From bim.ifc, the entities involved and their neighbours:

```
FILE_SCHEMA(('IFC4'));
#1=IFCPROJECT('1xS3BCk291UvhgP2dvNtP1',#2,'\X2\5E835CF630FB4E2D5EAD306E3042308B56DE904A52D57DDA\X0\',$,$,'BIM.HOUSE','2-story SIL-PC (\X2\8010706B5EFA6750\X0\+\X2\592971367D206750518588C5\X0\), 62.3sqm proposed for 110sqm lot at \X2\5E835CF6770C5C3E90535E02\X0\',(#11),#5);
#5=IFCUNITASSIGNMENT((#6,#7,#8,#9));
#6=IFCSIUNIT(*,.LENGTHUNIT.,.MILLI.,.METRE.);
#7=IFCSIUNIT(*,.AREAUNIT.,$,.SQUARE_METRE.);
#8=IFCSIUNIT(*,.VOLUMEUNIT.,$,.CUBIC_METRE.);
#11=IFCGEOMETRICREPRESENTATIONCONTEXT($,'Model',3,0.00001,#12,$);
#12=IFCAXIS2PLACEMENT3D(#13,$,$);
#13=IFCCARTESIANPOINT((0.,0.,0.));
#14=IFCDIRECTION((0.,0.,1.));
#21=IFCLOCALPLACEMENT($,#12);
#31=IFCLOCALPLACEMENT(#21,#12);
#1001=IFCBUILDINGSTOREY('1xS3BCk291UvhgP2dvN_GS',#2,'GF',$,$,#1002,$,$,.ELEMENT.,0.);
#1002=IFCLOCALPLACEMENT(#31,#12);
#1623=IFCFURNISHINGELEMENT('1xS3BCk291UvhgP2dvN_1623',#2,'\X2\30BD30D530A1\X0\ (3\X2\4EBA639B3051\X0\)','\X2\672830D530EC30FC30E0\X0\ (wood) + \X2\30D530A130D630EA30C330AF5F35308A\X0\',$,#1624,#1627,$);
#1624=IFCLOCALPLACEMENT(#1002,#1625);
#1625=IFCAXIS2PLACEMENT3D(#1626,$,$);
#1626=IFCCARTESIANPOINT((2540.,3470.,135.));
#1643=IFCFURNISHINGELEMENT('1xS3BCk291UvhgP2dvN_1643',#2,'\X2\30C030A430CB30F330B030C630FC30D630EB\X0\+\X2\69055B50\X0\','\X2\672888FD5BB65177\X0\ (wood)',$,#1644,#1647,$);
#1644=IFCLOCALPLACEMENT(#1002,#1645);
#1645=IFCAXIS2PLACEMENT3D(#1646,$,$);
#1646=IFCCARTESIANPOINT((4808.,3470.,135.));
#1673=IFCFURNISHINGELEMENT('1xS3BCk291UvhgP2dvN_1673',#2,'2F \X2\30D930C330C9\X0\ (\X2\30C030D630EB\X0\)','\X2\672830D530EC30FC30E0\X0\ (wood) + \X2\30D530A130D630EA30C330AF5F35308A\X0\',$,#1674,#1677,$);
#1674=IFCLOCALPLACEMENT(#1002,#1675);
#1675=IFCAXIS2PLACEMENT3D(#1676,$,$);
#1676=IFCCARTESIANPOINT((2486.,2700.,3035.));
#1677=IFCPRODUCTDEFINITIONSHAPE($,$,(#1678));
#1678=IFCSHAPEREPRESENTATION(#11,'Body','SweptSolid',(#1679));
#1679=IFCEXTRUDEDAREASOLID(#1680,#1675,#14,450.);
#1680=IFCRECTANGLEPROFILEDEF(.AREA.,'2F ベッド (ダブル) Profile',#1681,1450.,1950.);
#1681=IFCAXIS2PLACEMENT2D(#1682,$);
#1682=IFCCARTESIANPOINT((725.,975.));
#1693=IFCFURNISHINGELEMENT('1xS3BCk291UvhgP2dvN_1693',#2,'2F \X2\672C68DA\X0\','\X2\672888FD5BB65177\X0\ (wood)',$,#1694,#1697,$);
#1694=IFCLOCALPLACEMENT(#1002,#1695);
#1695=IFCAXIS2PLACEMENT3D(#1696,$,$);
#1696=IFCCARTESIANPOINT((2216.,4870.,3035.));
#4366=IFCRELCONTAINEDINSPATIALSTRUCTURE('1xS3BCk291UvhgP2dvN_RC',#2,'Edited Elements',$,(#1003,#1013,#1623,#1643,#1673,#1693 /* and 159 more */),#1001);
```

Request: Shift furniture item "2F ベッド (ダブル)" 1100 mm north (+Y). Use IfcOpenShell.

```python
import ifcopenshell
import ifcopenshell.api.geometry
import ifcopenshell.util.placement
import ifcopenshell.util.unit

model = ifcopenshell.open("bim.ifc")
unit_scale = ifcopenshell.util.unit.calculate_unit_scale(model)

item = model.by_guid("1xS3BCk291UvhgP2dvN_1673")
matrix = ifcopenshell.util.placement.get_local_placement(item.ObjectPlacement)
matrix[1, 3] += 1.1 / unit_scale
ifcopenshell.api.geometry.edit_object_placement(model, product=item, matrix=matrix, is_si=False)

print(ifcopenshell.util.placement.get_local_placement(item.ObjectPlacement).round(3) + 0.0)

model.write("bim_updated.ifc")
```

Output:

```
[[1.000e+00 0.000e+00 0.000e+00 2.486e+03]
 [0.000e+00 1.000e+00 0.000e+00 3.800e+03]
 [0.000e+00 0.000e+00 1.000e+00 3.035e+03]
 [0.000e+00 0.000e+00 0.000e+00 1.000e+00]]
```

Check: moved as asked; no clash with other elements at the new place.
